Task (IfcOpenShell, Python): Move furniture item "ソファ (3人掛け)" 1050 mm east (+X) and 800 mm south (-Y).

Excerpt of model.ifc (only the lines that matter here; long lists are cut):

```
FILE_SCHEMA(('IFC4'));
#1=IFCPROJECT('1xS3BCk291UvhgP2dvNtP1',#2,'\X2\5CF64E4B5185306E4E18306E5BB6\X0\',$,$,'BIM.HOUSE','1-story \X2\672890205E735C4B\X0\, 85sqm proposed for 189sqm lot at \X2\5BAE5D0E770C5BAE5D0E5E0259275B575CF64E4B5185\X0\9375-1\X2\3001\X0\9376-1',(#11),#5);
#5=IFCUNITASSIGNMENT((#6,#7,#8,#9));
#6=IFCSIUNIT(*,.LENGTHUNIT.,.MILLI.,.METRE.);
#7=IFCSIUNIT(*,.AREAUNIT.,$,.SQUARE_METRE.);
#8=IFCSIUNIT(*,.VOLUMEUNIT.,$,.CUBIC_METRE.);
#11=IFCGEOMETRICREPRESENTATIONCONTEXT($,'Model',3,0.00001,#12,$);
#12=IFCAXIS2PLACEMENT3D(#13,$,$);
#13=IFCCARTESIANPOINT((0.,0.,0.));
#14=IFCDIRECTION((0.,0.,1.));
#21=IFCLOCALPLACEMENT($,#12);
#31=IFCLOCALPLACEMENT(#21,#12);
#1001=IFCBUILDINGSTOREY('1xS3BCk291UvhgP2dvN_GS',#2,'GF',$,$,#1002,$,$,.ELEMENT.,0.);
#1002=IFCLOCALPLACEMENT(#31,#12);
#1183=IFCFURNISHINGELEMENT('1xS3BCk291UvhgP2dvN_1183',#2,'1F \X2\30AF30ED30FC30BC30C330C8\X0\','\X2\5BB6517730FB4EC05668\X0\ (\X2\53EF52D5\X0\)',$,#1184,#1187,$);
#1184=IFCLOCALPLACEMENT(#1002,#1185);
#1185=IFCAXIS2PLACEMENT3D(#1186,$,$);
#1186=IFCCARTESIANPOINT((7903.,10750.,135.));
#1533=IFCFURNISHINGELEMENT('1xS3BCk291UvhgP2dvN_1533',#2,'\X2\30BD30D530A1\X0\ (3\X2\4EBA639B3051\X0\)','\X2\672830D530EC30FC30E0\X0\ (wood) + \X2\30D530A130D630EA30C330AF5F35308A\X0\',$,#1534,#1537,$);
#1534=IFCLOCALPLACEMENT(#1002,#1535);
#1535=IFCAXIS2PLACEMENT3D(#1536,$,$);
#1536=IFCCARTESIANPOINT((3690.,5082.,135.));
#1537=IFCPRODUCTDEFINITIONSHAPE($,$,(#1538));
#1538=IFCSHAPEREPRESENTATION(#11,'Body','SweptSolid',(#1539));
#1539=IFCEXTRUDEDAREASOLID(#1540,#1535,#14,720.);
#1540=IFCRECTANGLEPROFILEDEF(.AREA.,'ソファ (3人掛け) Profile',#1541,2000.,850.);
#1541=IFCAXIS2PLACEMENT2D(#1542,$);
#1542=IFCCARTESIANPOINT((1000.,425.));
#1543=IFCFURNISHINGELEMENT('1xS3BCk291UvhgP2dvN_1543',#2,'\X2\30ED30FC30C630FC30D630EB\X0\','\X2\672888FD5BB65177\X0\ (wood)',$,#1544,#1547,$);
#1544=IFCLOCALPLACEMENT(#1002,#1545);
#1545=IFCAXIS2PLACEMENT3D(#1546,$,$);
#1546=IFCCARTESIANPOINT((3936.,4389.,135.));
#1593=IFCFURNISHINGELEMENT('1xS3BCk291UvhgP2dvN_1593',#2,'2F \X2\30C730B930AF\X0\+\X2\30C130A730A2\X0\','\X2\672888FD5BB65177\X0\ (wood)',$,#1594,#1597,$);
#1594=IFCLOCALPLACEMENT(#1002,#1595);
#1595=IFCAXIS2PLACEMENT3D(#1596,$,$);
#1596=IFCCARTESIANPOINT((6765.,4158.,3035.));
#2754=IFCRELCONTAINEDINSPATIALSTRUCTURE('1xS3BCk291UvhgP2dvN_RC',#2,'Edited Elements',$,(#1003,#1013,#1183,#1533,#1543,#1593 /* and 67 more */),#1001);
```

```python
import ifcopenshell
import ifcopenshell.api.geometry
import ifcopenshell.util.placement
import ifcopenshell.util.unit

model = ifcopenshell.open("model.ifc")
unit_scale = ifcopenshell.util.unit.calculate_unit_scale(model)

item = model.by_guid("1xS3BCk291UvhgP2dvN_1533")
matrix = ifcopenshell.util.placement.get_local_placement(item.ObjectPlacement)
matrix[0, 3] += 1.05 / unit_scale
matrix[1, 3] -= 0.8 / unit_scale
ifcopenshell.api.geometry.edit_object_placement(model, product=item, matrix=matrix, is_si=False)

print(ifcopenshell.util.placement.get_local_placement(item.ObjectPlacement).round(3) + 0.0)

model.write("model_edited.ifc")
```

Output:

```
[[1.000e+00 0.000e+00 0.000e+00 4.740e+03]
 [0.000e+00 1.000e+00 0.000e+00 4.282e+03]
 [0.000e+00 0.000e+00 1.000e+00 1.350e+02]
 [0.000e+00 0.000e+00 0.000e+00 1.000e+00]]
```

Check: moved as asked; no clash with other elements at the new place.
